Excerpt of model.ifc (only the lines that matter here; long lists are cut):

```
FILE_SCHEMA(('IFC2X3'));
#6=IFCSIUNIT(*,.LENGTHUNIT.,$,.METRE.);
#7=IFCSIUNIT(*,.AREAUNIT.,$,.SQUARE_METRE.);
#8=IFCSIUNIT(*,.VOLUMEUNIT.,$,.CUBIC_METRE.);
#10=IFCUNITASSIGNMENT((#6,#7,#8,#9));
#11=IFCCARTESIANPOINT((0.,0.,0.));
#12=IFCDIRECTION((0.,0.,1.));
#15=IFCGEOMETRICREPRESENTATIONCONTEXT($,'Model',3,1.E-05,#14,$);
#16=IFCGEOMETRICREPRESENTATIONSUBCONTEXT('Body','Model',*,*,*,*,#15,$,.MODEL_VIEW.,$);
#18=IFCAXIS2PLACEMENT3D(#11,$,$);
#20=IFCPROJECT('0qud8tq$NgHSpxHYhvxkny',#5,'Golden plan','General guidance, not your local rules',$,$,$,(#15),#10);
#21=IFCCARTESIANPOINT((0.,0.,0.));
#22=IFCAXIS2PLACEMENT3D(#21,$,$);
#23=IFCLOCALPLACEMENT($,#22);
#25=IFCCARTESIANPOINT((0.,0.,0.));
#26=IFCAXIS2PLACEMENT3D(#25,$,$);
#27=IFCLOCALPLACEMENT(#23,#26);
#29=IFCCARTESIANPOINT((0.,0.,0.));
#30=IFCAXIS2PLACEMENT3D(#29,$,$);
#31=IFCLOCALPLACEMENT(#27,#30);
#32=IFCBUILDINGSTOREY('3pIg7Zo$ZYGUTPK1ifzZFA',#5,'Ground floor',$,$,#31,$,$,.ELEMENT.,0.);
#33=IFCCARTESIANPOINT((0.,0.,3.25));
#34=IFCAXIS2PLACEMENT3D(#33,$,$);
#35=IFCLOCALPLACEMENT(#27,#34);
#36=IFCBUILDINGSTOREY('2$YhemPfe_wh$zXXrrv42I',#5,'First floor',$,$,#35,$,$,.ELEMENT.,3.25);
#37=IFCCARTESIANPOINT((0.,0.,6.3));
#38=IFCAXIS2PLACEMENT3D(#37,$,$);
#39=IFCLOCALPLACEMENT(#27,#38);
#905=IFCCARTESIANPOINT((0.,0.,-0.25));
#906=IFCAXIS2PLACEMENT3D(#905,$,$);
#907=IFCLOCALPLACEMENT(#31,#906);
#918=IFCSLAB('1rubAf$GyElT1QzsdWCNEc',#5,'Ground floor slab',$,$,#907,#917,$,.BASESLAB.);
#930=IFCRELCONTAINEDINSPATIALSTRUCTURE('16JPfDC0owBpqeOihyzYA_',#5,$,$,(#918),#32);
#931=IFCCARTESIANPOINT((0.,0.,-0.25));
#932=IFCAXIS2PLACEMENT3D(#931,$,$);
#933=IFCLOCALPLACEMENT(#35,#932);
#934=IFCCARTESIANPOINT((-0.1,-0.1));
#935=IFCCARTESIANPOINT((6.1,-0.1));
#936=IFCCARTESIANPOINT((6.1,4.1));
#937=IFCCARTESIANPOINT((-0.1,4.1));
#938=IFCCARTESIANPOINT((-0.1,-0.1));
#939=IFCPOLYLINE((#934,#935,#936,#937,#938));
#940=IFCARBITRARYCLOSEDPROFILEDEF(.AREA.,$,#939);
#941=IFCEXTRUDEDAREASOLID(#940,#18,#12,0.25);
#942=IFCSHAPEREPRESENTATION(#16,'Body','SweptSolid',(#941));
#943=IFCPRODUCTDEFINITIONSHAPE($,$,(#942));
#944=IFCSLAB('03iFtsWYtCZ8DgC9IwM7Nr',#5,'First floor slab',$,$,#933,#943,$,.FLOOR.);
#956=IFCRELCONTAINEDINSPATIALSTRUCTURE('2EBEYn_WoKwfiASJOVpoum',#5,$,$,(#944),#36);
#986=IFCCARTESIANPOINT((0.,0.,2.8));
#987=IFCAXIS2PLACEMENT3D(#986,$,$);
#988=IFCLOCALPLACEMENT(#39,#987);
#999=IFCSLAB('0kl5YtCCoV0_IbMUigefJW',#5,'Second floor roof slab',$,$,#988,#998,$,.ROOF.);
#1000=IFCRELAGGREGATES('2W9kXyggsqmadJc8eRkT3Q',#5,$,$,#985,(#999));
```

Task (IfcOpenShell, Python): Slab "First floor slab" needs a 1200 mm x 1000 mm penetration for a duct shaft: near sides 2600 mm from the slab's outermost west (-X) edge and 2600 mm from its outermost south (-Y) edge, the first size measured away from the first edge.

```python
import numpy as np
import ifcopenshell
import ifcopenshell.api.feature
import ifcopenshell.api.geometry
import ifcopenshell.api.root
import ifcopenshell.geom
import ifcopenshell.util.placement
import ifcopenshell.util.representation
import ifcopenshell.util.shape
import ifcopenshell.util.unit

model = ifcopenshell.open("model.ifc")
unit_scale = ifcopenshell.util.unit.calculate_unit_scale(model)
settings = ifcopenshell.geom.settings()


def volume(element):
    """Net volume in cubic metres, openings subtracted."""
    shape = ifcopenshell.geom.create_shape(settings, element)
    return ifcopenshell.util.shape.get_volume(shape.geometry)


slab = model.by_guid("03iFtsWYtCZ8DgC9IwM7Nr")
before = volume(slab)

# Extent in the slab's own axes, in metres. The edges named are its -X and -Y sides.
slab_shape = ifcopenshell.geom.create_shape(settings, slab)
vertices = ifcopenshell.util.shape.get_vertices(slab_shape.geometry)
x_min, y_min, bottom = vertices.min(axis=0)
top = vertices[:, 2].max()

opening = ifcopenshell.api.root.create_entity(model, ifc_class="IfcOpeningElement", name="Duct shaft opening")
context = ifcopenshell.util.representation.get_context(model, "Model", "Body", "MODEL_VIEW")
width, depth = 1.2, 1
outline = [(0.0, 0.0), (width, 0.0), (width, depth), (0.0, depth), (0.0, 0.0)]
# Overshoot both faces by 50 mm so the cut is clean.
shape = ifcopenshell.api.geometry.add_slab_representation(
    model, context=context, depth=top - bottom + 0.1, polyline=outline
)
ifcopenshell.api.geometry.assign_representation(model, product=opening, representation=shape)

matrix = ifcopenshell.util.placement.get_local_placement(slab.ObjectPlacement)
matrix[:, 3] = matrix @ np.append(np.array([x_min + 2.6, y_min + 2.6, bottom - 0.05]) / unit_scale, 1.0)
ifcopenshell.api.geometry.edit_object_placement(model, product=opening, matrix=matrix, is_si=False)
ifcopenshell.api.feature.add_feature(model, feature=opening, element=slab)

after = volume(slab)

print(f"slab volume {before:.3f} -> {after:.3f} m3")

model.write("model_updated.ifc")
```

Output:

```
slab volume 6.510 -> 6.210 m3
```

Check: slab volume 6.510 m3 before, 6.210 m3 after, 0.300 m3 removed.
